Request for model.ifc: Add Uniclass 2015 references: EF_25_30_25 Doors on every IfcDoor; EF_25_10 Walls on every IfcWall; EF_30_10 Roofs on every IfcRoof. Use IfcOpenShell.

First a look at what the model holds.

```python
import ifcopenshell

model = ifcopenshell.open("model.ifc")
print(model.schema)
print("classifications:", [c.Name for c in model.by_type("IfcClassification")])
for ifc_class in ("IfcDoor", "IfcRoof", "IfcStair", "IfcWall", "IfcWindow"):
    print(ifc_class, len(model.by_type(ifc_class)))
```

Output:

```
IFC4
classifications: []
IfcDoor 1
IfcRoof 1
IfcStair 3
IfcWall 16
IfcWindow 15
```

```python
import ifcopenshell
import ifcopenshell.api.classification

model = ifcopenshell.open("model.ifc")

system = ifcopenshell.api.classification.add_classification(model, classification="Uniclass 2015")

codes = {
    "IfcDoor": ("EF_25_30_25", "Doors"),
    "IfcWall": ("EF_25_10", "Walls"),
    "IfcRoof": ("EF_30_10", "Roofs"),
}
for ifc_class, (code, name) in codes.items():
    products = model.by_type(ifc_class)
    ifcopenshell.api.classification.add_reference(
        model, products=products, classification=system, identification=code, name=name
    )
    print(code, len(products))

model.write("model_rev.ifc")
```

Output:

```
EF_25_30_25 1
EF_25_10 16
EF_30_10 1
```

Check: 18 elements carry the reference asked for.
